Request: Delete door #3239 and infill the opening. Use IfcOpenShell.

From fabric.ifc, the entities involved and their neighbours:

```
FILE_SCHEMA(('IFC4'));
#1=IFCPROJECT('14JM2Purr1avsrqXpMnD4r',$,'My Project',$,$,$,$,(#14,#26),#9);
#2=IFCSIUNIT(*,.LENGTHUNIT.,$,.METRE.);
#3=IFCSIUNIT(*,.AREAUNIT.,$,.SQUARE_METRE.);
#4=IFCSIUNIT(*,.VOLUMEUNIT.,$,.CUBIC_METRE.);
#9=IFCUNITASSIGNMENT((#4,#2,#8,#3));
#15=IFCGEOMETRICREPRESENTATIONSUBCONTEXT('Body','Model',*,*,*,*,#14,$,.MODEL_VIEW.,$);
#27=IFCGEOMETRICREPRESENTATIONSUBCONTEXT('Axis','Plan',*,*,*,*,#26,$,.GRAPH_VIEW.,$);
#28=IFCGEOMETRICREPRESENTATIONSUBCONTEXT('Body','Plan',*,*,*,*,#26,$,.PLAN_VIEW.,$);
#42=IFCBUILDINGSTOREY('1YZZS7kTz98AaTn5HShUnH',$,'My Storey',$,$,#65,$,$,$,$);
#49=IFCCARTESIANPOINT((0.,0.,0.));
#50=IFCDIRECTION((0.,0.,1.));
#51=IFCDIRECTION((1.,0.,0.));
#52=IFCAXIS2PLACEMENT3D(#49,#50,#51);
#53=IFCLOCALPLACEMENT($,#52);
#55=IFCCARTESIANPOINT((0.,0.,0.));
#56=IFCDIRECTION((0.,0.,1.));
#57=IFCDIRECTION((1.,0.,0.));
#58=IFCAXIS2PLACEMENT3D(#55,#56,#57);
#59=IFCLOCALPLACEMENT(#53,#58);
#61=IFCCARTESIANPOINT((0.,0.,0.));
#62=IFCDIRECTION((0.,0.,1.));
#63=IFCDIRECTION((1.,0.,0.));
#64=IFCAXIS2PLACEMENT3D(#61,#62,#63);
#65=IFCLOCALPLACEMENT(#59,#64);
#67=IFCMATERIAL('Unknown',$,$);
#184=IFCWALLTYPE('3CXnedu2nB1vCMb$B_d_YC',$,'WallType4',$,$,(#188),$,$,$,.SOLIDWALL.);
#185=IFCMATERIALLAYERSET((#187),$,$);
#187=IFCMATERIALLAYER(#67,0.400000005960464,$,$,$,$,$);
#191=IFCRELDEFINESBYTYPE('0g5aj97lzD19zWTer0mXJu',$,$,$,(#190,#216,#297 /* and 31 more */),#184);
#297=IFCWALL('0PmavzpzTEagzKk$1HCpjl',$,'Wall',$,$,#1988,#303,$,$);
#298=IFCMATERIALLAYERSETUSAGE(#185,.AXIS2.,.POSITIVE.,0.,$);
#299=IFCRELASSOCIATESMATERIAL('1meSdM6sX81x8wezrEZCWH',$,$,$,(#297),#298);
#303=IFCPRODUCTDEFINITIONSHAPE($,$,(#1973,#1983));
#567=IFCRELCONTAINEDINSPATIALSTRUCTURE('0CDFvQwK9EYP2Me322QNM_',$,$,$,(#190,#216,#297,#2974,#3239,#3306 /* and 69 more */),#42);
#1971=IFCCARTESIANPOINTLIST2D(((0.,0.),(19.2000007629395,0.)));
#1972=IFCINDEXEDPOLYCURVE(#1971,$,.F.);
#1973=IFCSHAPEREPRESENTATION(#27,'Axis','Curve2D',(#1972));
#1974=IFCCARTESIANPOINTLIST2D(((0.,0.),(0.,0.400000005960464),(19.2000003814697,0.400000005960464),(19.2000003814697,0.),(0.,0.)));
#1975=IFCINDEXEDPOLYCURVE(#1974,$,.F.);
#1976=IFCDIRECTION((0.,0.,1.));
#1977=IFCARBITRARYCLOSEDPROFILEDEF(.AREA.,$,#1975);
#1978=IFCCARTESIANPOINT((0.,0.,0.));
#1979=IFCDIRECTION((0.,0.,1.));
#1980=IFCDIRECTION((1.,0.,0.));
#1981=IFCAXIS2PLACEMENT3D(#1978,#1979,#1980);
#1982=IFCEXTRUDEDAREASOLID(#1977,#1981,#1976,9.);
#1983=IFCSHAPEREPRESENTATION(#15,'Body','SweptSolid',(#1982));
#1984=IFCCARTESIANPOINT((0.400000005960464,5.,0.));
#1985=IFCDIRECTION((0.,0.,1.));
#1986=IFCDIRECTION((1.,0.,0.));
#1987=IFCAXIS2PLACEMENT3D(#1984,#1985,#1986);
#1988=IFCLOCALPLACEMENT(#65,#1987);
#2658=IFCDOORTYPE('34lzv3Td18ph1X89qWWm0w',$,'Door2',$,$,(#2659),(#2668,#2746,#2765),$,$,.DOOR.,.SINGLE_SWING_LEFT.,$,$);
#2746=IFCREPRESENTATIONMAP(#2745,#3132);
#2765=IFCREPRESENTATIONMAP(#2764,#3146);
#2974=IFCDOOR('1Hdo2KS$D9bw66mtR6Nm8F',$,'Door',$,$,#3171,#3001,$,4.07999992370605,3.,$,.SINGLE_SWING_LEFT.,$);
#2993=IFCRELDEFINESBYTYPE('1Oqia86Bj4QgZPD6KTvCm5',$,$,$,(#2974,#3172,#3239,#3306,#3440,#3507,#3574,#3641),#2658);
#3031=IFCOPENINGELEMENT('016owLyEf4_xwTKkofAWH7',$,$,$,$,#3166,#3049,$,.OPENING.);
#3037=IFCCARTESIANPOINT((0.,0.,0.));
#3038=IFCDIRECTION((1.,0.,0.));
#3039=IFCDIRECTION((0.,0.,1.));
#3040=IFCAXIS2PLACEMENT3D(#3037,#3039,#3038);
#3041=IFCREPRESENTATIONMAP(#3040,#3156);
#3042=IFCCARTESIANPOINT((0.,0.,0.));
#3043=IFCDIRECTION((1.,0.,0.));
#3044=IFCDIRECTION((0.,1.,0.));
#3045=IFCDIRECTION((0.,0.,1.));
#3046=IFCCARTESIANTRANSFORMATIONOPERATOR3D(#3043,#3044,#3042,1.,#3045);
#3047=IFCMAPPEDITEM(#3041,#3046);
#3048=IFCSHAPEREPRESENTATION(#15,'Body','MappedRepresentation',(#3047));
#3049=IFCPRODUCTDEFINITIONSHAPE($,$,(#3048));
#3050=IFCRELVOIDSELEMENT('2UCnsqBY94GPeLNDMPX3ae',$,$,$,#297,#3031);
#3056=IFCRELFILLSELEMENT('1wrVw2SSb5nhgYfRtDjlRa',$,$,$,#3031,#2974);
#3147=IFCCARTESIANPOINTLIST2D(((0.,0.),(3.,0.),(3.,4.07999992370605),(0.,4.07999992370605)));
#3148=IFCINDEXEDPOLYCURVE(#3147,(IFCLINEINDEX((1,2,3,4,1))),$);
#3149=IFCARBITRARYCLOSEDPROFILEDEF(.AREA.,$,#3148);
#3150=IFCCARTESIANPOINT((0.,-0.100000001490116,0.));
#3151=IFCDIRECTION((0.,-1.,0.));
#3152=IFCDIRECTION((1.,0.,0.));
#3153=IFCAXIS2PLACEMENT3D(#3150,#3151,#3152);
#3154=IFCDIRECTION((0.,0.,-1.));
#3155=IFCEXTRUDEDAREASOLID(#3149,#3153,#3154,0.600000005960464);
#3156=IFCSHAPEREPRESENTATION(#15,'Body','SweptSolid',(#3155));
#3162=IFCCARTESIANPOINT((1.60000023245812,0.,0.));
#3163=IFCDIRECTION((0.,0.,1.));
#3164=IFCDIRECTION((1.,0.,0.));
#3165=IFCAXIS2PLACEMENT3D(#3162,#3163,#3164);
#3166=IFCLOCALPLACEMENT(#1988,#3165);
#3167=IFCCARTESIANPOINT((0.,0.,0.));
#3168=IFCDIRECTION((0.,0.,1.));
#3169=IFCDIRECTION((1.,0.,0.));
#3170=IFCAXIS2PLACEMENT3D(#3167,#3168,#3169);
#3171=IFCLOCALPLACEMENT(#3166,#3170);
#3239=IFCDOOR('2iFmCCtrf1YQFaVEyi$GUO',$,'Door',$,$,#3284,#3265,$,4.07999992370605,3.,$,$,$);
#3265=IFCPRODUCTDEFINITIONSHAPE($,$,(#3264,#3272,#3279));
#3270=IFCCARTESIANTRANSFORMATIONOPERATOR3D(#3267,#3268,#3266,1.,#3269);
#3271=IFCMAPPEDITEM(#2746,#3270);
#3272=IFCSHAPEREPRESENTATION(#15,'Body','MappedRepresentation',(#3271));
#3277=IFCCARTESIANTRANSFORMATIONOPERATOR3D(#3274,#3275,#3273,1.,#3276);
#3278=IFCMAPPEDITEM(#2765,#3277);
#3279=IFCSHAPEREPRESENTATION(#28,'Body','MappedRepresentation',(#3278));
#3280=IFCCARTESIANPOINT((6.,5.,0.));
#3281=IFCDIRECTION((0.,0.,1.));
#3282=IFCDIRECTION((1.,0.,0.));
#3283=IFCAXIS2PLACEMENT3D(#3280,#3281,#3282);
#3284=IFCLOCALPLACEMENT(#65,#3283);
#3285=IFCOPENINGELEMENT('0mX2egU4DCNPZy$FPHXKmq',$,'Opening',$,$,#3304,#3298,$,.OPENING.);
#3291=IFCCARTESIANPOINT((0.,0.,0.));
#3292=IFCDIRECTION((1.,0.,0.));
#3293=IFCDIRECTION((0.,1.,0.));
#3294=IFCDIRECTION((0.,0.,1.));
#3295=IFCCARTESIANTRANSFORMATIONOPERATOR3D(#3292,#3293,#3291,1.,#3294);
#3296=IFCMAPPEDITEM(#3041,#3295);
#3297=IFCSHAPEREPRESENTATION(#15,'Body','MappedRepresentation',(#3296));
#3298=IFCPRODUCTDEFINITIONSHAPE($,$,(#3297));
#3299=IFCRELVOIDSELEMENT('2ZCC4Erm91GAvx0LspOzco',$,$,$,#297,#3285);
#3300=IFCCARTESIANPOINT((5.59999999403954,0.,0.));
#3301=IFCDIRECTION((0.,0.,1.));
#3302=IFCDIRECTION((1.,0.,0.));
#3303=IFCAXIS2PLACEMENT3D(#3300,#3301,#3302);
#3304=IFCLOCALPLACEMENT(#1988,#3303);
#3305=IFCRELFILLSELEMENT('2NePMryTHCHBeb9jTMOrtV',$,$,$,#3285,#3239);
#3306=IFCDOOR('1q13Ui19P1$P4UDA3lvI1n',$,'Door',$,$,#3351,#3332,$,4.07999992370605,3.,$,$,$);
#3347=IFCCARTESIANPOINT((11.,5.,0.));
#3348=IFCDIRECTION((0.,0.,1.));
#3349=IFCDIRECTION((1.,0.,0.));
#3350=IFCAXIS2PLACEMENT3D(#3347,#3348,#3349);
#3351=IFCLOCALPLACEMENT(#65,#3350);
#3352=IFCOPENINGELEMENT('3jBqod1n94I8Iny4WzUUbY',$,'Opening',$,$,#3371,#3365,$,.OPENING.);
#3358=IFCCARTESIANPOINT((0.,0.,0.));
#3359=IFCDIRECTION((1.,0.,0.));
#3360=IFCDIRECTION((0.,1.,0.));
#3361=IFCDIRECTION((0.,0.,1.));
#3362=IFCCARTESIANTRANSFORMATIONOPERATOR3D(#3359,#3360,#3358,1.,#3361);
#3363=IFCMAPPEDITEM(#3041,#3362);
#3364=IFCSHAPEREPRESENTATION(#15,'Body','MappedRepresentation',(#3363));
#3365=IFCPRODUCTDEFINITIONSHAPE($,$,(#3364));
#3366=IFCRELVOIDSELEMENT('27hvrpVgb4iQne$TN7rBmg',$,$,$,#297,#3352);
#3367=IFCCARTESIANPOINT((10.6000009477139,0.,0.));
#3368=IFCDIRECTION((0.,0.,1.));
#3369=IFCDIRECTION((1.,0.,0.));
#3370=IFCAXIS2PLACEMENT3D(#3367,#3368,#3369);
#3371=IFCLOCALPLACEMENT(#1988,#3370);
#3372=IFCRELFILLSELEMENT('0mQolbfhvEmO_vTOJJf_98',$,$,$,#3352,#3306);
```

```python
import ifcopenshell
import ifcopenshell.api.feature
import ifcopenshell.api.root
import ifcopenshell.geom
import ifcopenshell.util.shape

model = ifcopenshell.open("fabric.ifc")
settings = ifcopenshell.geom.settings()


def volume(element):
    """Net volume in cubic metres, openings subtracted."""
    shape = ifcopenshell.geom.create_shape(settings, element)
    return ifcopenshell.util.shape.get_volume(shape.geometry)


door = model.by_id(3239)
opening = door.FillsVoids[0].RelatingOpeningElement
wall = opening.VoidsElements[0].RelatingBuildingElement
before = volume(wall)

ifcopenshell.api.root.remove_product(model, product=door)
ifcopenshell.api.feature.remove_feature(model, feature=opening)

after = volume(wall)

print(f"wall volume {before:.3f} -> {after:.3f} m3")

model.write("fabric_v2.ifc")
```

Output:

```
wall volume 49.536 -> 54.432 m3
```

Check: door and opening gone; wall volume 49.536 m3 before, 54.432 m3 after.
